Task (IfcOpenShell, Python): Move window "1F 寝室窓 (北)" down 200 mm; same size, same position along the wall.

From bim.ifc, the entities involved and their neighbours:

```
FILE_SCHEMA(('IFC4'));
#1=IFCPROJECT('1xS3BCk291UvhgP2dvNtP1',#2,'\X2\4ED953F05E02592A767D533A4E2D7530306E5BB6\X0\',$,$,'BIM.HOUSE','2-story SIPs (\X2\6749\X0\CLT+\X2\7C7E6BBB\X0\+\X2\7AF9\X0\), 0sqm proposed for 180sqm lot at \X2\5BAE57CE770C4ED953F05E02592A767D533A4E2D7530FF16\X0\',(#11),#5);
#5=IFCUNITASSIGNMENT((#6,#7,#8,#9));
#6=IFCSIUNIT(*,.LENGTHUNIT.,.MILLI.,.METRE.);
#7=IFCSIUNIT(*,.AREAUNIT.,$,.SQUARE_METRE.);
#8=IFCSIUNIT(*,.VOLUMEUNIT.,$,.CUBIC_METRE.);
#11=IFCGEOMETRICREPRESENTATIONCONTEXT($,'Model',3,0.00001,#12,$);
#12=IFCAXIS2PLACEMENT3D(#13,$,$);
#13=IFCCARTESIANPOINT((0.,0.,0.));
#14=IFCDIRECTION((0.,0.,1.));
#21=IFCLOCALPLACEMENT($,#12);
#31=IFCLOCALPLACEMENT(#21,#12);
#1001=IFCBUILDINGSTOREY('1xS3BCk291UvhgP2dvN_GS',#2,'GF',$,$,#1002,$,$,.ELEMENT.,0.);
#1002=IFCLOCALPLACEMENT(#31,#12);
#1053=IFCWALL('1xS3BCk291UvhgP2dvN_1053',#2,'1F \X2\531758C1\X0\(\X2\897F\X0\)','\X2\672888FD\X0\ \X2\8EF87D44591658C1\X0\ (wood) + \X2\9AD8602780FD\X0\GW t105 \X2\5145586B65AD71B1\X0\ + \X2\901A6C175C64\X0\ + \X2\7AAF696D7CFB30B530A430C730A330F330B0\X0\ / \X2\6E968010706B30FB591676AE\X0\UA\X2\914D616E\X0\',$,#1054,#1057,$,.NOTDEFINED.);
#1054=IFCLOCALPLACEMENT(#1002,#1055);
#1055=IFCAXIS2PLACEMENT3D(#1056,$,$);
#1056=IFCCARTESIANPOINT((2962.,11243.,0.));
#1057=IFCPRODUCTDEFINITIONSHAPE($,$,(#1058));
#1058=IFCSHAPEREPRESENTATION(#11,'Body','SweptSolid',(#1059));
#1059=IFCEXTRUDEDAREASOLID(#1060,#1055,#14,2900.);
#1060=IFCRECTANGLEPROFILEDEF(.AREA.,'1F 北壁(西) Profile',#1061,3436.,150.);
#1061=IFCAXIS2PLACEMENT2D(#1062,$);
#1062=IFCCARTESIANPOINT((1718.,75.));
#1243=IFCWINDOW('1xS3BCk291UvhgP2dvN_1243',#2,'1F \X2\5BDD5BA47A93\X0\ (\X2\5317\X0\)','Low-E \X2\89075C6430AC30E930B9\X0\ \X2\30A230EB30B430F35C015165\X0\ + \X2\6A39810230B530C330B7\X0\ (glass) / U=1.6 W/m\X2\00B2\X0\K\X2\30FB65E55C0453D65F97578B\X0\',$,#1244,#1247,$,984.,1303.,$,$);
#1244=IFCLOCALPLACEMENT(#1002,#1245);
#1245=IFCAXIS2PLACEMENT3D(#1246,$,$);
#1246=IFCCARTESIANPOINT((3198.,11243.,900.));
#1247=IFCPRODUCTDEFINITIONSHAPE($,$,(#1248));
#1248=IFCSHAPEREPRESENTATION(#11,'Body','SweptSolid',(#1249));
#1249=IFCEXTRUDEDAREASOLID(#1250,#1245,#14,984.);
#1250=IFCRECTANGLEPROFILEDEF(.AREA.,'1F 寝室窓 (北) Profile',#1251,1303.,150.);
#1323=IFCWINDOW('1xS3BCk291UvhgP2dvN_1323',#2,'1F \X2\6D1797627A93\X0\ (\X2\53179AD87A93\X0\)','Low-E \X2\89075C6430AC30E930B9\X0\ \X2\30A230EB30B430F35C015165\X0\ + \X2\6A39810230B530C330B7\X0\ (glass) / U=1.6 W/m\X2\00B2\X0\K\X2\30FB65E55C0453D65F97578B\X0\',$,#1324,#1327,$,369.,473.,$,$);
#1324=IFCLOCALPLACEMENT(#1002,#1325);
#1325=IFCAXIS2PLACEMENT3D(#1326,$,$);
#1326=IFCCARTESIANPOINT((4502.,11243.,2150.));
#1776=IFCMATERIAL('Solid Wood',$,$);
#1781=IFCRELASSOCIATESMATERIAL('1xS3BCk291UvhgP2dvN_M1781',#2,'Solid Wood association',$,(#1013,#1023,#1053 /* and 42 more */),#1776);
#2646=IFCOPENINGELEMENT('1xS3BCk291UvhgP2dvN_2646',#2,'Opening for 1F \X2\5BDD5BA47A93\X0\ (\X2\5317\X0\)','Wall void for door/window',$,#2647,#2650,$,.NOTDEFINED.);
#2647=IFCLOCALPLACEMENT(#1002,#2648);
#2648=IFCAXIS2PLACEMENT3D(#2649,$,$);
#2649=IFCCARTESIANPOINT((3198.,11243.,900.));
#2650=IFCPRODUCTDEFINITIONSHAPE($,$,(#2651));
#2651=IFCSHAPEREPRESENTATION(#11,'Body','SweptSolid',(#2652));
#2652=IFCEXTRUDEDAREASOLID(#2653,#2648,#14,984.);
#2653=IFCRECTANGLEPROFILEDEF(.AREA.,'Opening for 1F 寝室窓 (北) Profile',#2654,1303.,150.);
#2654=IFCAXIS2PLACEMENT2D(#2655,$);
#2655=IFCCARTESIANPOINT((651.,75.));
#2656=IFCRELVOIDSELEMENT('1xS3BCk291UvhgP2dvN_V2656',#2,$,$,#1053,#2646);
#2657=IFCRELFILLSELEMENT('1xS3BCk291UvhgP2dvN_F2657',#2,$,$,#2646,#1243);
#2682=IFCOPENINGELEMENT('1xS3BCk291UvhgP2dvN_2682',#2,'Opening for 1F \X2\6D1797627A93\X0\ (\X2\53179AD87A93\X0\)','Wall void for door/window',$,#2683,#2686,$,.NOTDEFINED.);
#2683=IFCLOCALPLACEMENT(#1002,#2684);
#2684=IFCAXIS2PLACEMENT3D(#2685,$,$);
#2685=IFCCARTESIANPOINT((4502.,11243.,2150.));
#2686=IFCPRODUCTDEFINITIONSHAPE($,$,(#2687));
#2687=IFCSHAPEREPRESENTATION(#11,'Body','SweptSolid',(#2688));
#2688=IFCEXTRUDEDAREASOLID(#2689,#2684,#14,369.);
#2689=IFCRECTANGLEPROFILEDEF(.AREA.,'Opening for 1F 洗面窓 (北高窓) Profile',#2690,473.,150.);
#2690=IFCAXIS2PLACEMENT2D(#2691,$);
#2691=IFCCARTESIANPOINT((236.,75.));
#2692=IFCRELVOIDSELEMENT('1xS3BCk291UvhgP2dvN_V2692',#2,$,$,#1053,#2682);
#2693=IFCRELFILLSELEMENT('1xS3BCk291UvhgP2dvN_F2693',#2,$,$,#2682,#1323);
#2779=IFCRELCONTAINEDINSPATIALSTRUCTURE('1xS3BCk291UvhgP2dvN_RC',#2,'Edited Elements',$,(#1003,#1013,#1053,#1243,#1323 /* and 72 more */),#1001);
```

```python
import numpy as np
import ifcopenshell
import ifcopenshell.api.geometry
import ifcopenshell.util.placement
import ifcopenshell.util.unit

model = ifcopenshell.open("bim.ifc")
unit_scale = ifcopenshell.util.unit.calculate_unit_scale(model)

window = model.by_guid("1xS3BCk291UvhgP2dvN_1243")
opening = window.FillsVoids[0].RelatingOpeningElement
dz = -0.2 / unit_scale

shift = np.array([0.0, 0.0, dz])
# The window is not placed relative to its opening, so move both.
for product in (opening, window):
    matrix = ifcopenshell.util.placement.get_local_placement(product.ObjectPlacement)
    matrix[:3, 3] += shift
    ifcopenshell.api.geometry.edit_object_placement(model, product=product, matrix=matrix, is_si=False)

print(f"moved by {dz * unit_scale:+.3f} m")

model.write("bim_edited.ifc")
```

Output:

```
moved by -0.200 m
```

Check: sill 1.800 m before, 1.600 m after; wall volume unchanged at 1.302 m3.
